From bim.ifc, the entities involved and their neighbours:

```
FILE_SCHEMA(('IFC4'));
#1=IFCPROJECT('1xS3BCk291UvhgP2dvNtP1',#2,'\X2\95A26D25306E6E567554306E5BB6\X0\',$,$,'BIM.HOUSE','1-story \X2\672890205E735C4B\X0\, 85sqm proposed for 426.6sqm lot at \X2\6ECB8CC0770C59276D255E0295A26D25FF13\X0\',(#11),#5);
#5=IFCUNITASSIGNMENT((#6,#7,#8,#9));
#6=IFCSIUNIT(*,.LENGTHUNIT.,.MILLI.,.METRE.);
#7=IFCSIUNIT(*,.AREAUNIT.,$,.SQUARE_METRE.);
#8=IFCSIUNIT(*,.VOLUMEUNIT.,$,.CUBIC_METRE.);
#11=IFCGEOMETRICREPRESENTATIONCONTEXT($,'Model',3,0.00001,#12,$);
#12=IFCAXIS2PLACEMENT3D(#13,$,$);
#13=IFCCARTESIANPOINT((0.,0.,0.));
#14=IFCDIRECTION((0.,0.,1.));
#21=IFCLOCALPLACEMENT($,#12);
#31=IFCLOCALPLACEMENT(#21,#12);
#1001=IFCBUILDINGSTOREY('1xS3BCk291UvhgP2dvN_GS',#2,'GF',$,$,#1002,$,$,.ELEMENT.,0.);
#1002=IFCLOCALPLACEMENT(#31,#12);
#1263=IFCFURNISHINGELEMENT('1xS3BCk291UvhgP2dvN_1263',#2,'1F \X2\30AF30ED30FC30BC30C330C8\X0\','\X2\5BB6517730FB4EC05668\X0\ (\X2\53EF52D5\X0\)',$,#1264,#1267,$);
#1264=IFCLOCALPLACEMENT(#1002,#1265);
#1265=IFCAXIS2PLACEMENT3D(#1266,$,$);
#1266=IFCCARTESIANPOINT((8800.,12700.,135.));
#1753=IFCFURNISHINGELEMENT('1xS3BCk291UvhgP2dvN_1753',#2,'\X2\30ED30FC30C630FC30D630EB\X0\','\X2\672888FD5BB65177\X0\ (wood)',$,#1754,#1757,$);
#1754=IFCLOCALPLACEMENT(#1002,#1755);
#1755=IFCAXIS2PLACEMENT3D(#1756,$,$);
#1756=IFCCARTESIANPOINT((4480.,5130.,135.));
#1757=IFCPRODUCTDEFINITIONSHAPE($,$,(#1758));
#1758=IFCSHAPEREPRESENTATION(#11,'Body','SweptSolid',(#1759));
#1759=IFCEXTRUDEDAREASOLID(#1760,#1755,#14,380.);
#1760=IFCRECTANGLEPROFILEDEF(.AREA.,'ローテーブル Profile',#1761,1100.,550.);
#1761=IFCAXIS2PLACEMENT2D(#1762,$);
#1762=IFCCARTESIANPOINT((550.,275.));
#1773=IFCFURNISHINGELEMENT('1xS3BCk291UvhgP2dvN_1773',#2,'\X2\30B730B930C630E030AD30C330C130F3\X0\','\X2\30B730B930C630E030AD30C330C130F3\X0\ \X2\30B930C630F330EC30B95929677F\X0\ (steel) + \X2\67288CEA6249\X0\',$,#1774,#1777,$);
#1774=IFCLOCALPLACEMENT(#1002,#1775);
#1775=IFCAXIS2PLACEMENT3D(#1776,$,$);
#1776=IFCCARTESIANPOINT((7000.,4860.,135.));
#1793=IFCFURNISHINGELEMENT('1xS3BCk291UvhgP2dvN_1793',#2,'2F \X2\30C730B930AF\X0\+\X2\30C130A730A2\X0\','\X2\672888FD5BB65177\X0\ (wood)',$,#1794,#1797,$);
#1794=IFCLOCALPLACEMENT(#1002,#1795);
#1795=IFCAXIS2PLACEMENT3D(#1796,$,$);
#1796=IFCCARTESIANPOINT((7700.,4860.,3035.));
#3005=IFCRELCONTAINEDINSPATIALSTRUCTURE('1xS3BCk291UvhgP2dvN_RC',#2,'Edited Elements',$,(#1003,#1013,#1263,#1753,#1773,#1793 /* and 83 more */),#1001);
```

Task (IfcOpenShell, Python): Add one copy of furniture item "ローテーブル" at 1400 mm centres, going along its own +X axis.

```python
import ifcopenshell
import ifcopenshell.api.geometry
import ifcopenshell.api.root
import ifcopenshell.util.element
import ifcopenshell.util.placement
import ifcopenshell.util.unit

model = ifcopenshell.open("bim.ifc")
unit_scale = ifcopenshell.util.unit.calculate_unit_scale(model)


def reuse_history(source, copy):
    """copy_class also copies each property set's owner history, people and application; keep the originals."""
    for rel in copy.IsDefinedBy:
        if rel.is_a("IfcRelDefinesByProperties") and (history := rel.RelatingPropertyDefinition.OwnerHistory):
            rel.RelatingPropertyDefinition.OwnerHistory = source.OwnerHistory
            ifcopenshell.util.element.remove_deep2(model, history)


source = model.by_guid("1xS3BCk291UvhgP2dvN_1753")
base = ifcopenshell.util.placement.get_local_placement(source.ObjectPlacement)
step = base[:3, 0] * 1.4 / unit_scale

for i in range(1, 2):
    copy = ifcopenshell.api.root.copy_class(model, product=source)
    copy.Representation = ifcopenshell.util.element.copy_deep(
        model, source.Representation, exclude=["IfcGeometricRepresentationContext", "IfcRepresentationMap"]
    )
    reuse_history(source, copy)
    matrix = base.copy()
    matrix[:3, 3] += i * step
    print("added at", matrix[:3, 3].round(3) + 0.0)
    ifcopenshell.api.geometry.edit_object_placement(model, product=copy, matrix=matrix, is_si=False)

model.write("bim_updated.ifc")
```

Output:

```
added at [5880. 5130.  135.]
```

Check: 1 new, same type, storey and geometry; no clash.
